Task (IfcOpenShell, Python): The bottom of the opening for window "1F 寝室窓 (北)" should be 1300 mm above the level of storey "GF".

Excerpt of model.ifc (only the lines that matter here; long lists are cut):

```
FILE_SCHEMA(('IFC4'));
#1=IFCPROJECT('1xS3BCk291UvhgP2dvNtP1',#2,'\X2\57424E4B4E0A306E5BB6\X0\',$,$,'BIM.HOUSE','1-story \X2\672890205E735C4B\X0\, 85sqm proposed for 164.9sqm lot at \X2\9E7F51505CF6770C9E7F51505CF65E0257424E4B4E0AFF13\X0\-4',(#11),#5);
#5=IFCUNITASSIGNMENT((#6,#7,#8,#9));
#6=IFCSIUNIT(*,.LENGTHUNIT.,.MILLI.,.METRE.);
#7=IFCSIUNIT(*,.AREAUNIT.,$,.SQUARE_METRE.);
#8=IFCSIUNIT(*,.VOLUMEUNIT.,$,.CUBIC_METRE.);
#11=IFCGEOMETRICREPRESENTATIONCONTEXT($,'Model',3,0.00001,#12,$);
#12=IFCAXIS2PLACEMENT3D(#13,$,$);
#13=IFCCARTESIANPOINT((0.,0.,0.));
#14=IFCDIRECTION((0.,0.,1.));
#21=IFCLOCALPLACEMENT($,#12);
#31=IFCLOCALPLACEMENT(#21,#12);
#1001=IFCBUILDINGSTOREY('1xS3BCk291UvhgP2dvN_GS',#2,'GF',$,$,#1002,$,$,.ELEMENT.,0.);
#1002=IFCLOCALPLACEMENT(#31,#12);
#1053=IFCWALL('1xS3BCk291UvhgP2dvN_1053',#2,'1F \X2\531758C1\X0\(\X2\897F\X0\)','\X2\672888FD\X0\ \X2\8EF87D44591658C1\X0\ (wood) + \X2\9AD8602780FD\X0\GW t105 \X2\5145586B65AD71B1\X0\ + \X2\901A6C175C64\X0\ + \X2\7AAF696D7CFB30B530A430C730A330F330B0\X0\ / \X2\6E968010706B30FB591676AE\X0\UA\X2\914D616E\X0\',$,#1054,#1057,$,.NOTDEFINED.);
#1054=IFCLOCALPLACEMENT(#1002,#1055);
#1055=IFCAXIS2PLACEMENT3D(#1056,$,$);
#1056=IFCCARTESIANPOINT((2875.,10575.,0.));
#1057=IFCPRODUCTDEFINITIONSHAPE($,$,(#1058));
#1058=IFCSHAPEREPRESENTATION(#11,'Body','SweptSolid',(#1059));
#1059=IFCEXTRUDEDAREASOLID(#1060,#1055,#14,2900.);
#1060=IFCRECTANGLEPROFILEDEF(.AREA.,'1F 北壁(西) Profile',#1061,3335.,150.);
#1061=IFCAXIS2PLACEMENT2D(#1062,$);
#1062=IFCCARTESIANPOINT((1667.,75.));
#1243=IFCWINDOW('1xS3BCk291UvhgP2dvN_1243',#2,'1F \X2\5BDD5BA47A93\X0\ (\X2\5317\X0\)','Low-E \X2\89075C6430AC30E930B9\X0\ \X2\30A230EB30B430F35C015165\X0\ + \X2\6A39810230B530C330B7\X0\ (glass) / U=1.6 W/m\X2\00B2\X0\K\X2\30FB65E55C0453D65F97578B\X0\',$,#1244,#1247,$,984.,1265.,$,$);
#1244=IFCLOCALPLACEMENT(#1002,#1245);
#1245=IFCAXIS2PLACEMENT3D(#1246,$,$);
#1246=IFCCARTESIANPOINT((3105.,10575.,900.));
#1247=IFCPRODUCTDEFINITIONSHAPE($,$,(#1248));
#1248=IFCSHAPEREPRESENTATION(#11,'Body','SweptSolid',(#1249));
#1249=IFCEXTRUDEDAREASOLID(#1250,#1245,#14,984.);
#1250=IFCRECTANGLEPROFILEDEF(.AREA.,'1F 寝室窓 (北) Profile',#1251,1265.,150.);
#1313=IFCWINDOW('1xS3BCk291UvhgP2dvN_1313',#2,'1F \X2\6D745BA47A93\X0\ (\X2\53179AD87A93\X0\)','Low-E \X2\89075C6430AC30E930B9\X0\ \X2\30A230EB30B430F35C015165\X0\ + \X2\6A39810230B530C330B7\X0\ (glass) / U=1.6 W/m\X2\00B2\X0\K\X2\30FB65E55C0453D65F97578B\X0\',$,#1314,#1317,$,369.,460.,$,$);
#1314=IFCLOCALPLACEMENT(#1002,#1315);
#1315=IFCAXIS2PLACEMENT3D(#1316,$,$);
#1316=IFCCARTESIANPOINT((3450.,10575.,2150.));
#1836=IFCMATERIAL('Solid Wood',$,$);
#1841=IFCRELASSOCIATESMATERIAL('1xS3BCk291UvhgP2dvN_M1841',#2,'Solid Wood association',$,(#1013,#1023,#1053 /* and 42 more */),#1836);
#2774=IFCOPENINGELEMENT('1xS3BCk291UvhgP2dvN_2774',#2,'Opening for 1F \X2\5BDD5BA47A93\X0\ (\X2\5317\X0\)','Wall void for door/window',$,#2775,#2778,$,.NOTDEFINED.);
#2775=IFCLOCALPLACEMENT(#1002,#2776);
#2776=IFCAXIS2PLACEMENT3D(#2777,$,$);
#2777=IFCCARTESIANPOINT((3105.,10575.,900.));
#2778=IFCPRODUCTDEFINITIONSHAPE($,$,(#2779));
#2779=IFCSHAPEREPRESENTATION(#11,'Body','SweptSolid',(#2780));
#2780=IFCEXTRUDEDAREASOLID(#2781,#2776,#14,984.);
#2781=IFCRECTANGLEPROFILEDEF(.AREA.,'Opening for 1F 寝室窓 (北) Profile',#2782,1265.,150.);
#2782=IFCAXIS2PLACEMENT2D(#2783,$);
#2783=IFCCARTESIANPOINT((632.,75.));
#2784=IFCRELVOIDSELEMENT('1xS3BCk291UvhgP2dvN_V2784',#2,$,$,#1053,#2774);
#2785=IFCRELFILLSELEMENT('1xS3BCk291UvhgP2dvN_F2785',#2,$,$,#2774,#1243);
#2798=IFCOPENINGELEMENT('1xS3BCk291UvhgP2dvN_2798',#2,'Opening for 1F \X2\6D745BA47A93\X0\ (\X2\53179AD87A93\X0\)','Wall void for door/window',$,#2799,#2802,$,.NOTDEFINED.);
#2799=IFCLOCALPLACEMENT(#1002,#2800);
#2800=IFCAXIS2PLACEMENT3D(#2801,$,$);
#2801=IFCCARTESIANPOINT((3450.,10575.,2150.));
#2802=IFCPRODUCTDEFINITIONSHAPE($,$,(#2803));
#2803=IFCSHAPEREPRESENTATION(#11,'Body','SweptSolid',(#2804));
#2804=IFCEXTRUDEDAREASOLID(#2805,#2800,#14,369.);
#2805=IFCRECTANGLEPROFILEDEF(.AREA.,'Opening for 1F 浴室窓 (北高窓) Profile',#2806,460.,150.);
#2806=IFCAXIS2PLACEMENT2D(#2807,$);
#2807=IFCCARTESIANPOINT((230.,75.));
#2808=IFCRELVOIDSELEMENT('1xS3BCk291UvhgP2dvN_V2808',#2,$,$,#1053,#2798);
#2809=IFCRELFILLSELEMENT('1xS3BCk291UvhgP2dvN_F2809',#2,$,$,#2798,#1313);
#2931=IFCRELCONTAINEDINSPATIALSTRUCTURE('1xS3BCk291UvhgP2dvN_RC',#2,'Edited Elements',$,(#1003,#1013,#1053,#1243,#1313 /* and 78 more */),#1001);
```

```python
import numpy as np
import ifcopenshell
import ifcopenshell.api.geometry
import ifcopenshell.geom
import ifcopenshell.util.element
import ifcopenshell.util.placement
import ifcopenshell.util.shape
import ifcopenshell.util.unit

model = ifcopenshell.open("model.ifc")
unit_scale = ifcopenshell.util.unit.calculate_unit_scale(model)

window = model.by_guid("1xS3BCk291UvhgP2dvN_1243")
opening = window.FillsVoids[0].RelatingOpeningElement
storey = ifcopenshell.util.element.get_container(window, ifc_class="IfcBuildingStorey")
level = ifcopenshell.util.placement.get_local_placement(storey.ObjectPlacement)[2, 3]

# The opening's origin need not be at the sill, so measure its lowest point.
shape = ifcopenshell.geom.create_shape(ifcopenshell.geom.settings(), opening)
bottom = ifcopenshell.util.shape.get_shape_bottom_elevation(shape, shape.geometry) / unit_scale
dz = level + 1300.0 - bottom

shift = np.array([0.0, 0.0, dz])
# The window is not placed relative to its opening, so move both.
for product in (opening, window):
    matrix = ifcopenshell.util.placement.get_local_placement(product.ObjectPlacement)
    matrix[:3, 3] += shift
    ifcopenshell.api.geometry.edit_object_placement(model, product=product, matrix=matrix, is_si=False)

print(f"moved by {dz * unit_scale:+.3f} m")

model.write("model_rev.ifc")
```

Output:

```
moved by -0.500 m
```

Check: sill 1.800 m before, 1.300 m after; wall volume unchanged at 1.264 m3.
